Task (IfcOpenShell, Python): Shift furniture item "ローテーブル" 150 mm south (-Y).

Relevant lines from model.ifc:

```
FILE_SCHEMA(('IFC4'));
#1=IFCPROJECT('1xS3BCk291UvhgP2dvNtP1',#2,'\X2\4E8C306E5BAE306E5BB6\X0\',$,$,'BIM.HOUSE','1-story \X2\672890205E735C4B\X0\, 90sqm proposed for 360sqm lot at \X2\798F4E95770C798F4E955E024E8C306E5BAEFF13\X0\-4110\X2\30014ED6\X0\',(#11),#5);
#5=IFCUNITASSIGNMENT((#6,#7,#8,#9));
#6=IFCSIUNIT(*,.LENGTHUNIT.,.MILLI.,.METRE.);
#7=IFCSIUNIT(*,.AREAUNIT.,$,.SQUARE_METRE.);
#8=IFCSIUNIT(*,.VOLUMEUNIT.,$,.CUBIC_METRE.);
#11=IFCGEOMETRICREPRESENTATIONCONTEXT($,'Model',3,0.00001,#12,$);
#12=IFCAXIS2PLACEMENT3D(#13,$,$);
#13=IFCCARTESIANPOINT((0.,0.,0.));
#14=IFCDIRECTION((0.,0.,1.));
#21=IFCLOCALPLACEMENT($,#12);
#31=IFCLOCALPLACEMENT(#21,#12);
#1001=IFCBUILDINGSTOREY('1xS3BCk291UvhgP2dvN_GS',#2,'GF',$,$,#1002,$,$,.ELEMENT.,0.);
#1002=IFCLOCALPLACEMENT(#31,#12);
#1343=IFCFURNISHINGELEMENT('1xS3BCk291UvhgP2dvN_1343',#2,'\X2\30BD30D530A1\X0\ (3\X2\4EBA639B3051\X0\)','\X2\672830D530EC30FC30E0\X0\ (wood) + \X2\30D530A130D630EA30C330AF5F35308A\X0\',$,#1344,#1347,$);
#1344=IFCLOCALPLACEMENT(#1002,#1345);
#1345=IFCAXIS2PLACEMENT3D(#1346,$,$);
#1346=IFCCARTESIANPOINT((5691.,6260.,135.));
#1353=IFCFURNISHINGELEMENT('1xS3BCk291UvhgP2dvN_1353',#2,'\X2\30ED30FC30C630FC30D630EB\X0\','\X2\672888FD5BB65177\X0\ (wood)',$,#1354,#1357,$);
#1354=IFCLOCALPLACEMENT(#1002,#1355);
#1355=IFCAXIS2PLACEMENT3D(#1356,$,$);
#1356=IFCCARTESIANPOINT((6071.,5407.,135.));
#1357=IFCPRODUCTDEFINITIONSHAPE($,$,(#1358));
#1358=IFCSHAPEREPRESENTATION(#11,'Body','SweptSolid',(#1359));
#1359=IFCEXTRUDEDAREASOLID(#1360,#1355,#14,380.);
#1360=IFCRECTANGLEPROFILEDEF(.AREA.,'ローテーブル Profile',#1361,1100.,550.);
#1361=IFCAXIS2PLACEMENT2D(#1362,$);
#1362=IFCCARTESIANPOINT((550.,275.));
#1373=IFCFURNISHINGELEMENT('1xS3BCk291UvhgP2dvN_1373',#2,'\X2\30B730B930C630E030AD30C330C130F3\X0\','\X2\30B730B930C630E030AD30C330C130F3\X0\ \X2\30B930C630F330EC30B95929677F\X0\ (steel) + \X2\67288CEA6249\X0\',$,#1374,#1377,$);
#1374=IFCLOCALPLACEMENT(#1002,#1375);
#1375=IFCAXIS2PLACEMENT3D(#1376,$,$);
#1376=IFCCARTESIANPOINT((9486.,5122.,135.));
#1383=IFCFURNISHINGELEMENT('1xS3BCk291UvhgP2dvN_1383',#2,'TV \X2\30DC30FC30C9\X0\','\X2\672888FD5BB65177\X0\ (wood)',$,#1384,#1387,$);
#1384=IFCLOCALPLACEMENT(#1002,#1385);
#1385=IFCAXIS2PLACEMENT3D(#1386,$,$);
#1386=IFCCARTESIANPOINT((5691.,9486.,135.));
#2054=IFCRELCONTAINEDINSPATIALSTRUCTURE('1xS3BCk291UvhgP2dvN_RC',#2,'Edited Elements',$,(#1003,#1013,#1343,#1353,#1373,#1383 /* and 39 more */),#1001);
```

```python
import ifcopenshell
import ifcopenshell.api.geometry
import ifcopenshell.util.placement
import ifcopenshell.util.unit

model = ifcopenshell.open("model.ifc")
unit_scale = ifcopenshell.util.unit.calculate_unit_scale(model)

item = model.by_guid("1xS3BCk291UvhgP2dvN_1353")
matrix = ifcopenshell.util.placement.get_local_placement(item.ObjectPlacement)
matrix[1, 3] -= 0.15 / unit_scale
ifcopenshell.api.geometry.edit_object_placement(model, product=item, matrix=matrix, is_si=False)

print(ifcopenshell.util.placement.get_local_placement(item.ObjectPlacement).round(3) + 0.0)

model.write("model_updated.ifc")
```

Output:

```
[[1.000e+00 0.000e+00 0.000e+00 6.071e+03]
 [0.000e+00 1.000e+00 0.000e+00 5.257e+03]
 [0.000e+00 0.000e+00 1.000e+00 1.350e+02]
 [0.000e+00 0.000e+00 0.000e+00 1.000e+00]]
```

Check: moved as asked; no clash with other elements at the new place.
